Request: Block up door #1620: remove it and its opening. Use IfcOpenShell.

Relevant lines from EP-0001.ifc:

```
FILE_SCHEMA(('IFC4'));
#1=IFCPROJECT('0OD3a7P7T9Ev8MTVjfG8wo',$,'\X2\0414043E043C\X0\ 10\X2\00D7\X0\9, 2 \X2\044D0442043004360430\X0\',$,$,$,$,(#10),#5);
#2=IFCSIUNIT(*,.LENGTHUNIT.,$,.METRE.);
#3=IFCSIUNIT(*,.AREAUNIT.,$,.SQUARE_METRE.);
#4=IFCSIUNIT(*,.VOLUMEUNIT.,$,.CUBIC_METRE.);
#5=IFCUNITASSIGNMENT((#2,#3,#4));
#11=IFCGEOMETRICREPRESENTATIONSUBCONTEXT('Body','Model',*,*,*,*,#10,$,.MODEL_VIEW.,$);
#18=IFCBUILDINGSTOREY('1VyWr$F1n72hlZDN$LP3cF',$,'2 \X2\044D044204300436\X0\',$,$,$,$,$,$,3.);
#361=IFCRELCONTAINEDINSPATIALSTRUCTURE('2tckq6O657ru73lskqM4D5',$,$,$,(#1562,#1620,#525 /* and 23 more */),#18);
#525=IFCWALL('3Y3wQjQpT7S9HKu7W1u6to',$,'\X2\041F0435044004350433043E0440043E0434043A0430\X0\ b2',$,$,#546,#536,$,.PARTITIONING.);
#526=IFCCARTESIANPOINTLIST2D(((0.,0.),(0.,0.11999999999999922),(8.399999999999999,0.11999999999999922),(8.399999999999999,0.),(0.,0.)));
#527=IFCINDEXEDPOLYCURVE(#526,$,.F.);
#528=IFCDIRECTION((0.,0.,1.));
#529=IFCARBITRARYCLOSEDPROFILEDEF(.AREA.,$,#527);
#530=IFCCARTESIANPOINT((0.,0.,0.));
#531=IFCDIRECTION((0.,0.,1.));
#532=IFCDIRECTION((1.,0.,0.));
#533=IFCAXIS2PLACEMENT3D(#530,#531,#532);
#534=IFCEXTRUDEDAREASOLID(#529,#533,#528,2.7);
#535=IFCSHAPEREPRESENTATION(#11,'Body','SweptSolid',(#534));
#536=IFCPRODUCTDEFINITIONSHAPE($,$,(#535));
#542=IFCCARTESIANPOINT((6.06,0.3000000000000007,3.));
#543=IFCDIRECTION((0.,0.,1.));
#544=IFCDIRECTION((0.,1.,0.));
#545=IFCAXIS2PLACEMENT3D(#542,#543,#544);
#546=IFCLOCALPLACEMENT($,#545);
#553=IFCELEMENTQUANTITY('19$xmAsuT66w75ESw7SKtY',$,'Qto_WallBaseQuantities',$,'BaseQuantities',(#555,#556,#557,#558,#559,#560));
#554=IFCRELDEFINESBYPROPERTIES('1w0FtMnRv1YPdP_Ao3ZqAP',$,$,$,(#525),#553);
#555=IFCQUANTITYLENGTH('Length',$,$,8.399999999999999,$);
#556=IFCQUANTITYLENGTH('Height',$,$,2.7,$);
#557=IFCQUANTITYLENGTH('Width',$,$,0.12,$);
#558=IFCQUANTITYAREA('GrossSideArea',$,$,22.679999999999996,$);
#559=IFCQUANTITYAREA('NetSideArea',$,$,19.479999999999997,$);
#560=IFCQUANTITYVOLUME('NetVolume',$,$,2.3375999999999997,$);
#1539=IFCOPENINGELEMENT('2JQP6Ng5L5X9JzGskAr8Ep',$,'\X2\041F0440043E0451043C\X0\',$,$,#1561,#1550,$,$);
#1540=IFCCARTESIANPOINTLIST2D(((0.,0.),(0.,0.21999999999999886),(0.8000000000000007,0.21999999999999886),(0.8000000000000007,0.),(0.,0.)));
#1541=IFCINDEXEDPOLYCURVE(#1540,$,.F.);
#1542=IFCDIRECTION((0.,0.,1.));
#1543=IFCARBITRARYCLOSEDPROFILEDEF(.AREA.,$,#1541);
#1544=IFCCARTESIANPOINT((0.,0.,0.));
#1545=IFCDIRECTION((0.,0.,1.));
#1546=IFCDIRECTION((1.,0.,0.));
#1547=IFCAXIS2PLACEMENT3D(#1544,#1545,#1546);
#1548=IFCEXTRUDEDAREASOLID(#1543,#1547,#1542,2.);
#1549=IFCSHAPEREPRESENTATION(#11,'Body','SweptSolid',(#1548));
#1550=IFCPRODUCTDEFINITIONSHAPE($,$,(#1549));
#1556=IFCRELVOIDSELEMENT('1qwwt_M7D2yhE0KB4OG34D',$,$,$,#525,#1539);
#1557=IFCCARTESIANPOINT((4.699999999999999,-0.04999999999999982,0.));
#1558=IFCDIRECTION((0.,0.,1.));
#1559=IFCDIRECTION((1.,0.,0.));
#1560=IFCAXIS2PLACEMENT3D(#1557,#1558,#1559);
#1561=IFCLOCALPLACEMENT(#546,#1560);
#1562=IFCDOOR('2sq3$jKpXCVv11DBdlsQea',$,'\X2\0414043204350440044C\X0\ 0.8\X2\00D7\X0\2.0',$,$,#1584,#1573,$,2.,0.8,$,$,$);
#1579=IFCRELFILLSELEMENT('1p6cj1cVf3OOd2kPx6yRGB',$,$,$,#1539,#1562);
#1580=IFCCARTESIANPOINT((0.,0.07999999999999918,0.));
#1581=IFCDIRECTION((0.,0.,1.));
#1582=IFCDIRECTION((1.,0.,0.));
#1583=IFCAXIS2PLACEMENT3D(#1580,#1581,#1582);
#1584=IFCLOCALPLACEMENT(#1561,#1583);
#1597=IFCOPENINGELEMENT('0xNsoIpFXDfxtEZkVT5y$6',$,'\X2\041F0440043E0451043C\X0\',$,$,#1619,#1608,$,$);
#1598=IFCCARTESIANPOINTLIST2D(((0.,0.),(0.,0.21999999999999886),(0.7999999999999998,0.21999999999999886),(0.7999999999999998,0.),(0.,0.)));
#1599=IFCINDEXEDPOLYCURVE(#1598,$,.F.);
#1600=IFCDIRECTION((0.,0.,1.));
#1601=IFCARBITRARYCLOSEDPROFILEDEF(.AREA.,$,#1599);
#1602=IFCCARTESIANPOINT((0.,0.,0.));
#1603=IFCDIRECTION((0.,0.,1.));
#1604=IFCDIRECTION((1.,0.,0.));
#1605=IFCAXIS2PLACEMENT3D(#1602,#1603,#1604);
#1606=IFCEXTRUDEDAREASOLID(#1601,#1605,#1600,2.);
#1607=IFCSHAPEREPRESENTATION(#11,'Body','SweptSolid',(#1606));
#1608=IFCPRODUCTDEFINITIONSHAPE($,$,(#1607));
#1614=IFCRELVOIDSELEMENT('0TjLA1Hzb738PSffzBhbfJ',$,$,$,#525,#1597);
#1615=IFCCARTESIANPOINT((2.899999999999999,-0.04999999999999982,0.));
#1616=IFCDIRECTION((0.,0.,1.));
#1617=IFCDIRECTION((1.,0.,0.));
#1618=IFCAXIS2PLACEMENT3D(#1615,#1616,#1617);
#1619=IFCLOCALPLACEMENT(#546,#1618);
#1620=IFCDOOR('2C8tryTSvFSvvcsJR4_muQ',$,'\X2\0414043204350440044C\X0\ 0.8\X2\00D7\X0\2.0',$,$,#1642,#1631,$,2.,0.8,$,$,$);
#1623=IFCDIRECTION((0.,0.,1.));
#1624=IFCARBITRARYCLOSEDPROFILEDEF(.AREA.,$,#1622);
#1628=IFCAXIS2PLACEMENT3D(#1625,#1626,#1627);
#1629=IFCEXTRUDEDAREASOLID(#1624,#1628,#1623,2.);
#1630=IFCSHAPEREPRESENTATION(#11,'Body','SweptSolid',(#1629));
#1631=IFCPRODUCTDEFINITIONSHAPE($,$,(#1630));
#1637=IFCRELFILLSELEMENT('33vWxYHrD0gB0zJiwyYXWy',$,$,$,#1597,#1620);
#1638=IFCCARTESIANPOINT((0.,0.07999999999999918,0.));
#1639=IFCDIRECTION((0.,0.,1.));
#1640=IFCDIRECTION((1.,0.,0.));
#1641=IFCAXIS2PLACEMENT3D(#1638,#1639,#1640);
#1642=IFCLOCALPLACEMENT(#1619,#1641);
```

```python
import ifcopenshell
import ifcopenshell.api.feature
import ifcopenshell.api.pset
import ifcopenshell.api.root
import ifcopenshell.geom
import ifcopenshell.util.element
import ifcopenshell.util.shape
import ifcopenshell.util.unit

model = ifcopenshell.open("EP-0001.ifc")
area_scale = ifcopenshell.util.unit.calculate_unit_scale(model, "AREAUNIT")
volume_scale = ifcopenshell.util.unit.calculate_unit_scale(model, "VOLUMEUNIT")
settings = ifcopenshell.geom.settings()


def volume(element):
    """Net volume in cubic metres, openings subtracted."""
    shape = ifcopenshell.geom.create_shape(settings, element)
    return ifcopenshell.util.shape.get_volume(shape.geometry)


door = model.by_guid("2C8tryTSvFSvvcsJR4_muQ")
opening = door.FillsVoids[0].RelatingOpeningElement
wall = opening.VoidsElements[0].RelatingBuildingElement
before = volume(wall)

ifcopenshell.api.root.remove_product(model, product=door)
ifcopenshell.api.feature.remove_feature(model, feature=opening)

after = volume(wall)
thickness = 0.12  # wall thickness in metres

# Update the wall's stored quantities.
qto = model.by_id(ifcopenshell.util.element.get_pset(wall, "Qto_WallBaseQuantities", should_inherit=False)["id"])
ifcopenshell.api.pset.edit_qto(model, qto=qto, properties={
    "NetSideArea": after / thickness / area_scale,
    "NetVolume": after / volume_scale,
})

print(f"wall volume {before:.3f} -> {after:.3f} m3")

model.write("EP-0001_updated.ifc")
```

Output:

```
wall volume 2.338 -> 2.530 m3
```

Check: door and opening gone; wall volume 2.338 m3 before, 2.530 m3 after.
